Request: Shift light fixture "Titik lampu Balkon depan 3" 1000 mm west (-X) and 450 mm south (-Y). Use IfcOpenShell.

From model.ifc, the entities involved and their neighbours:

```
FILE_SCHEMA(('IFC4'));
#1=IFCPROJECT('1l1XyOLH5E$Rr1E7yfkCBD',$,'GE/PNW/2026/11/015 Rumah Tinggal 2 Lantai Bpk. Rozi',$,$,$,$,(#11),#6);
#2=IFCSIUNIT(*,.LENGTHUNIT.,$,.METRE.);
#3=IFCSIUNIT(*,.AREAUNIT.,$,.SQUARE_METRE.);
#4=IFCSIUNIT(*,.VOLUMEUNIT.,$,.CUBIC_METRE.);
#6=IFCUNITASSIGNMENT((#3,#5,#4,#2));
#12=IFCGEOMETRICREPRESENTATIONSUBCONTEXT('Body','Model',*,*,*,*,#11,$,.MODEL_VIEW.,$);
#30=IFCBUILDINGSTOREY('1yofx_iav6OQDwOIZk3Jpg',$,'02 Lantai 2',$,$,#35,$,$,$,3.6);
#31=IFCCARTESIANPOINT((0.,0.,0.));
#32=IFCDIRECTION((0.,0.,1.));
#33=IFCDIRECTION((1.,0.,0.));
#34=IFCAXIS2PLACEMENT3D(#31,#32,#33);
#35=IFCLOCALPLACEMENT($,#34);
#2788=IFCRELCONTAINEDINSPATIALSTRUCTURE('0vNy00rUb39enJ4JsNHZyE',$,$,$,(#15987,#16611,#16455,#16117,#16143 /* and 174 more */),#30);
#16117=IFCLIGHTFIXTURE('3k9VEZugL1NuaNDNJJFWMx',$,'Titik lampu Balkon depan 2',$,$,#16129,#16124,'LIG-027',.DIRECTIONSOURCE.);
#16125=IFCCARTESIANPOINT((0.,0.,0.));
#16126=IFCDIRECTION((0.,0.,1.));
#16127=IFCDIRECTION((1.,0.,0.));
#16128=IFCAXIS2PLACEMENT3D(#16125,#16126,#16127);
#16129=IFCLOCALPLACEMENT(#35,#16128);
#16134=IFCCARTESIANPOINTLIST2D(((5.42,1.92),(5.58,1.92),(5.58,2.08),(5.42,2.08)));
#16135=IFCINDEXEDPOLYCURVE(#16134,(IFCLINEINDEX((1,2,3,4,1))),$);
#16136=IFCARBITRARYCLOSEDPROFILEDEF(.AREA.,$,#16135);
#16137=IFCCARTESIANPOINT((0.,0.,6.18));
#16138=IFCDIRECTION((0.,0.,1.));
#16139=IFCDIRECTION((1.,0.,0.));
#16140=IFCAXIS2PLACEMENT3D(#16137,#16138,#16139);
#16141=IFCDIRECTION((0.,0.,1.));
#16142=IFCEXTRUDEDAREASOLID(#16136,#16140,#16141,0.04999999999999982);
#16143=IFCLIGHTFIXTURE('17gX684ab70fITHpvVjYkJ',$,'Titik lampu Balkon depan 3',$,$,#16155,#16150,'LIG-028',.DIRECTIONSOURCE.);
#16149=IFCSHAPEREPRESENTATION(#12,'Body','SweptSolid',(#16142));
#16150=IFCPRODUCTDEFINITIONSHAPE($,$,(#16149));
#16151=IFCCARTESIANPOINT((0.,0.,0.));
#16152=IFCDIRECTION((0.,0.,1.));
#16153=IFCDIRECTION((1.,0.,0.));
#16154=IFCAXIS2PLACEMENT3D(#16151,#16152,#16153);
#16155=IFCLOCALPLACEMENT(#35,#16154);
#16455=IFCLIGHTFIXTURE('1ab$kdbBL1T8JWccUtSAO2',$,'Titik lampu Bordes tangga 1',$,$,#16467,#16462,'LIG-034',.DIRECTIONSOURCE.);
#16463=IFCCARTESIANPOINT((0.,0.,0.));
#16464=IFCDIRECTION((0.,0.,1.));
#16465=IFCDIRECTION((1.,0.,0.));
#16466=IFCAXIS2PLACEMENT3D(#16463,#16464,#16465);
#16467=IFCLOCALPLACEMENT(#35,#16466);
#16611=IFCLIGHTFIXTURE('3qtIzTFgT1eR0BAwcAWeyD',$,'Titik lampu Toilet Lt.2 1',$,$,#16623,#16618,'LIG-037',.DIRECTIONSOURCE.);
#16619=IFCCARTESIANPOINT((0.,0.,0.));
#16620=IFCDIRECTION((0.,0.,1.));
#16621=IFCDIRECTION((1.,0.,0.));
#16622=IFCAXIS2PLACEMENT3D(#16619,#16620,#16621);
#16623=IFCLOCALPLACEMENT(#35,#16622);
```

```python
import ifcopenshell
import ifcopenshell.api.geometry
import ifcopenshell.util.placement

model = ifcopenshell.open("model.ifc")

item = model.by_guid("17gX684ab70fITHpvVjYkJ")
matrix = ifcopenshell.util.placement.get_local_placement(item.ObjectPlacement)
matrix[0, 3] -= 1.0
matrix[1, 3] -= 0.45
ifcopenshell.api.geometry.edit_object_placement(model, product=item, matrix=matrix, is_si=False)

print(ifcopenshell.util.placement.get_local_placement(item.ObjectPlacement).round(3) + 0.0)

model.write("model_v2.ifc")
```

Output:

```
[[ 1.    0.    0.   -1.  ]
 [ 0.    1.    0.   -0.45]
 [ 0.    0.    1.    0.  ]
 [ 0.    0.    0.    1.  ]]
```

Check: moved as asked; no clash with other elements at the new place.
